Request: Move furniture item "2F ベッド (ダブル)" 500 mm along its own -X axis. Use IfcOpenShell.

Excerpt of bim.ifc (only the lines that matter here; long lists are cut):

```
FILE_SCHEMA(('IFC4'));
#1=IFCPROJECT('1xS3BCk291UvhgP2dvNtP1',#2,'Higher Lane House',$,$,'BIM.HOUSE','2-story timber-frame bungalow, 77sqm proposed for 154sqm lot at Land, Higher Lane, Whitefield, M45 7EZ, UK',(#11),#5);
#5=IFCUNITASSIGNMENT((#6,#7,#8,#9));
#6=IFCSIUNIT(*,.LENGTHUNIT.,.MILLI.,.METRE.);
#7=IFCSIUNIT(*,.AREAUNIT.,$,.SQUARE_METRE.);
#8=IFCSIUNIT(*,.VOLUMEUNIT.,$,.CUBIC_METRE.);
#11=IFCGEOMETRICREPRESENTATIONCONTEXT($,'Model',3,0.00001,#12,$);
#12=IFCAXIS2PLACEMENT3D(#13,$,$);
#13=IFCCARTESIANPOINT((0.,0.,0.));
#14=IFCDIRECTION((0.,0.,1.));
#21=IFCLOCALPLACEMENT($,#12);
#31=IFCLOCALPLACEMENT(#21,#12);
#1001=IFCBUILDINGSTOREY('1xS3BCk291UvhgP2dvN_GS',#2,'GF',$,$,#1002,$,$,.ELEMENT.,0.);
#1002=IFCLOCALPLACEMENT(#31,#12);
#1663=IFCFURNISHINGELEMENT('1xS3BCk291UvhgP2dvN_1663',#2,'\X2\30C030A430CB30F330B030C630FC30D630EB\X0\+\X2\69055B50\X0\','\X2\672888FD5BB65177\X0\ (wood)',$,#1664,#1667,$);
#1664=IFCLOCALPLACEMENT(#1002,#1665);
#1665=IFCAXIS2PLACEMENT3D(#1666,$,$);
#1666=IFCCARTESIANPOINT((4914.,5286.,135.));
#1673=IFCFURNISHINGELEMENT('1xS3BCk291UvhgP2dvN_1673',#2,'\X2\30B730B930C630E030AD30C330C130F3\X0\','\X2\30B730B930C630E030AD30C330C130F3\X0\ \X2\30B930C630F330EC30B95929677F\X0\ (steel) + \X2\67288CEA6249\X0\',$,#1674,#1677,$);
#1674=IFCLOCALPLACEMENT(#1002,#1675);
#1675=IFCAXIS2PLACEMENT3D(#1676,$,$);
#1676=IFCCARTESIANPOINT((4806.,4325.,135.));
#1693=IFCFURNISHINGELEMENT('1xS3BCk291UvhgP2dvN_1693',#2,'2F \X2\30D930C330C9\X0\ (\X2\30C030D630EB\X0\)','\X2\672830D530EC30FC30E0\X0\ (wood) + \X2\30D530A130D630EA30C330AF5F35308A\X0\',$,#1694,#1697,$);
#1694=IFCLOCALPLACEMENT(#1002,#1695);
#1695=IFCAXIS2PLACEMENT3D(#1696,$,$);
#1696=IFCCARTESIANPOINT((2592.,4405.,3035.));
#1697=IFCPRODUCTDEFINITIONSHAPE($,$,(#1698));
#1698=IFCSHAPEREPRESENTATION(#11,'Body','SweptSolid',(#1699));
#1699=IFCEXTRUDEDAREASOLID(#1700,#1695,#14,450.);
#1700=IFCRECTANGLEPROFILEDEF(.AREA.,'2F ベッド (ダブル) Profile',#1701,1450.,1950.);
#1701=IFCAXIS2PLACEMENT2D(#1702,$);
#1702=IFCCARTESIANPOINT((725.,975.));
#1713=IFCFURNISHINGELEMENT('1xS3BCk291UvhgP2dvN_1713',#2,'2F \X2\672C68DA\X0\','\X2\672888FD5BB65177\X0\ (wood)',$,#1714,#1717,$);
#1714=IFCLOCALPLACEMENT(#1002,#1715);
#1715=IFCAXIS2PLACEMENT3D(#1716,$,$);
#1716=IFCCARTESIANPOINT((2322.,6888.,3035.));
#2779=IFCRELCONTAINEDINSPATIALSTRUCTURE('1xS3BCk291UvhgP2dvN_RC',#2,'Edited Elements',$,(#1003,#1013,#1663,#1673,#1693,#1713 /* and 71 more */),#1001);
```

```python
import ifcopenshell
import ifcopenshell.api.geometry
import ifcopenshell.util.placement

model = ifcopenshell.open("bim.ifc")

item = model.by_guid("1xS3BCk291UvhgP2dvN_1693")
matrix = ifcopenshell.util.placement.get_local_placement(item.ObjectPlacement)
matrix[:3, 3] -= matrix[:3, 0] * 500.0
ifcopenshell.api.geometry.edit_object_placement(model, product=item, matrix=matrix, is_si=False)

print(ifcopenshell.util.placement.get_local_placement(item.ObjectPlacement).round(3) + 0.0)

model.write("bim_edited.ifc")
```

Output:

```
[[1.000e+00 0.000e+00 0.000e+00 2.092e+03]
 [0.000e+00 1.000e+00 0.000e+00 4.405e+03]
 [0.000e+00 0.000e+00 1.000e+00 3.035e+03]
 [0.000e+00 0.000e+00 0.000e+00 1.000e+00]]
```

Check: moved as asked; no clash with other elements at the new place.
